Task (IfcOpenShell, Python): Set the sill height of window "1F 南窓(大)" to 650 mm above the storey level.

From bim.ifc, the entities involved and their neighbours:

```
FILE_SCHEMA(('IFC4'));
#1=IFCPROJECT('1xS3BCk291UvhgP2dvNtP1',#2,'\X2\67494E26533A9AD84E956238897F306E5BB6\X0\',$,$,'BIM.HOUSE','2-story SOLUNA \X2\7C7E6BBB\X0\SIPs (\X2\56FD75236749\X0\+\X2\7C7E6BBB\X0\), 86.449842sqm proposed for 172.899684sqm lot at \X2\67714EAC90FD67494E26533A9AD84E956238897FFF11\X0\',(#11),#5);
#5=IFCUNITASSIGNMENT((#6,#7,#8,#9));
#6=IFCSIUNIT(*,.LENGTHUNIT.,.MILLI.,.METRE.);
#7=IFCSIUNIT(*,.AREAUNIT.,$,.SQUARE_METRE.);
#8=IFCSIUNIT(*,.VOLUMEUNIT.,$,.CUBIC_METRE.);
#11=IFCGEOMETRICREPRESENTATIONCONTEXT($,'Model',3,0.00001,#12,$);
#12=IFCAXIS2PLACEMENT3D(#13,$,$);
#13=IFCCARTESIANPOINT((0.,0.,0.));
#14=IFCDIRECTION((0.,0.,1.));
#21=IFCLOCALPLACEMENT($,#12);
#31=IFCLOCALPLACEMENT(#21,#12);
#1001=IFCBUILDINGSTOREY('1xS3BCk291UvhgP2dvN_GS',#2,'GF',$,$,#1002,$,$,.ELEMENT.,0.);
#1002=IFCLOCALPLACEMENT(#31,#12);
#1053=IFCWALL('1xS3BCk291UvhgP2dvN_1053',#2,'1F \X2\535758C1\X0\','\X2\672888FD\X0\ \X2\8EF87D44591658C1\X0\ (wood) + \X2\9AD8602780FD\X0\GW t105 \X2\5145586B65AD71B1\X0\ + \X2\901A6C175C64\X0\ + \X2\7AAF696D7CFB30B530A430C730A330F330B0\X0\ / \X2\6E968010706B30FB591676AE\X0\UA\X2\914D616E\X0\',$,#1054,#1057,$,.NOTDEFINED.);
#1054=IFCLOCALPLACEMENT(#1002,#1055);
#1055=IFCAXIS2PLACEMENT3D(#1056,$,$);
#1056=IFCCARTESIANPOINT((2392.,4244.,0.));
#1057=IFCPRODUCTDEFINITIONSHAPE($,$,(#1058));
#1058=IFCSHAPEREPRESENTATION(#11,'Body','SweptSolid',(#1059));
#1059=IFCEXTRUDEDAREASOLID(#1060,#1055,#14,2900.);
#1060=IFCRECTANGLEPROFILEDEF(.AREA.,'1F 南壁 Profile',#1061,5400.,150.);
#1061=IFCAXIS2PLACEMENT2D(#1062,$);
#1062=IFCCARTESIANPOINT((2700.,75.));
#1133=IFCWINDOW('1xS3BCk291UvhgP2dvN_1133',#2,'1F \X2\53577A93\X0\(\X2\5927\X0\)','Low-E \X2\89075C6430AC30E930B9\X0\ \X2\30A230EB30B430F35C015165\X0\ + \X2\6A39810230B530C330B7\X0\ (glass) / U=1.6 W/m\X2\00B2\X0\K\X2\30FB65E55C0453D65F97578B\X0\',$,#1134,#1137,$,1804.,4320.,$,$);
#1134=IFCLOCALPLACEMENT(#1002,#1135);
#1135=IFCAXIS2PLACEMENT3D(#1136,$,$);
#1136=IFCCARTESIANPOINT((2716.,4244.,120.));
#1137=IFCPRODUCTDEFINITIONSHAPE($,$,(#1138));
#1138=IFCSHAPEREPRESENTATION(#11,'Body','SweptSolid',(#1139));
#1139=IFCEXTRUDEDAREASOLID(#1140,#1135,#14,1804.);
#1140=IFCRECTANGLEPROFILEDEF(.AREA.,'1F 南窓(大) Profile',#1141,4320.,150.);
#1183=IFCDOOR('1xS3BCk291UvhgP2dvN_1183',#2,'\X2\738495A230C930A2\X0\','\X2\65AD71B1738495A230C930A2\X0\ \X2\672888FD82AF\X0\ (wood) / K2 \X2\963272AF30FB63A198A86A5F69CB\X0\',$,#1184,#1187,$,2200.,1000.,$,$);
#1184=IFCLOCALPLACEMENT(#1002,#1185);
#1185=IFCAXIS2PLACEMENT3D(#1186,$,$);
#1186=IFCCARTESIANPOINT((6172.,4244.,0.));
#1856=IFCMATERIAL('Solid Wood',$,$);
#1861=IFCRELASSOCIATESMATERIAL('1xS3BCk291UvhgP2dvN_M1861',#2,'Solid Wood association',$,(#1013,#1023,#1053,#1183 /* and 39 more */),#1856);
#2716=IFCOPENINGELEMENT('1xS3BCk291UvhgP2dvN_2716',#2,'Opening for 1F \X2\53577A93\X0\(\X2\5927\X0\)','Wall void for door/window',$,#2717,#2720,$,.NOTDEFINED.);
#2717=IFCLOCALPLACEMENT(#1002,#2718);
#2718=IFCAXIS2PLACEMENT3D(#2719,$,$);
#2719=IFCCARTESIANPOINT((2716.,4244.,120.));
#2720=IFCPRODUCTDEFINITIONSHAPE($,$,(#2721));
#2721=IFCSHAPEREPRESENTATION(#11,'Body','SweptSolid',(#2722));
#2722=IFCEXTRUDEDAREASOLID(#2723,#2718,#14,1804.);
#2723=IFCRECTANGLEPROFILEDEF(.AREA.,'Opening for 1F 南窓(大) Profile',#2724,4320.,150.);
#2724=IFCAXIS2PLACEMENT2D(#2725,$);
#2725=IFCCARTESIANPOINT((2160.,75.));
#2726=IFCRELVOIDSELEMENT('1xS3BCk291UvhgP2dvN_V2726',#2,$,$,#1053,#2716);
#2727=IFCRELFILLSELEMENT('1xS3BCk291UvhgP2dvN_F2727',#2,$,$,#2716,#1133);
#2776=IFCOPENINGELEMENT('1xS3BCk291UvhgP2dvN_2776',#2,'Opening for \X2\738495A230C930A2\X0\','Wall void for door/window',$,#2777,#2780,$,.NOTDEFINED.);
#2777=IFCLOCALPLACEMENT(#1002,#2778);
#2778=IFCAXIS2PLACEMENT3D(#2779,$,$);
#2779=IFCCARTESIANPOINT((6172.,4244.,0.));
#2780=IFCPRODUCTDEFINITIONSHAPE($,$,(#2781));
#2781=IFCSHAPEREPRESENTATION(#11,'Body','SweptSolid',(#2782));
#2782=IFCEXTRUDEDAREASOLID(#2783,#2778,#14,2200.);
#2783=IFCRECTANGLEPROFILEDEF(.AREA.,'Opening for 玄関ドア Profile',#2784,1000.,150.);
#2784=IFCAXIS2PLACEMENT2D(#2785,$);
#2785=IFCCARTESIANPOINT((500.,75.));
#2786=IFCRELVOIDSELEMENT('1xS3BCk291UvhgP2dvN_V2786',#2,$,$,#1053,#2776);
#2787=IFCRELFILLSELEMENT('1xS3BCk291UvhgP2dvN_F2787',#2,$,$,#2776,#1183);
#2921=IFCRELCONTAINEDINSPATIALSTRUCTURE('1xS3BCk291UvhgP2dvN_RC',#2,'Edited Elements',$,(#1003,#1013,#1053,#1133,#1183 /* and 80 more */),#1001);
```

```python
import numpy as np
import ifcopenshell
import ifcopenshell.api.geometry
import ifcopenshell.geom
import ifcopenshell.util.element
import ifcopenshell.util.placement
import ifcopenshell.util.shape
import ifcopenshell.util.unit

model = ifcopenshell.open("bim.ifc")
unit_scale = ifcopenshell.util.unit.calculate_unit_scale(model)

window = model.by_guid("1xS3BCk291UvhgP2dvN_1133")
opening = window.FillsVoids[0].RelatingOpeningElement
storey = ifcopenshell.util.element.get_container(window, ifc_class="IfcBuildingStorey")
level = ifcopenshell.util.placement.get_local_placement(storey.ObjectPlacement)[2, 3]

# The opening's origin need not be at the sill, so measure its lowest point.
shape = ifcopenshell.geom.create_shape(ifcopenshell.geom.settings(), opening)
bottom = ifcopenshell.util.shape.get_shape_bottom_elevation(shape, shape.geometry) / unit_scale
dz = level + 0.65 / unit_scale - bottom

shift = np.array([0.0, 0.0, dz])
# The window is not placed relative to its opening, so move both.
for product in (opening, window):
    matrix = ifcopenshell.util.placement.get_local_placement(product.ObjectPlacement)
    matrix[:3, 3] += shift
    ifcopenshell.api.geometry.edit_object_placement(model, product=product, matrix=matrix, is_si=False)

print(f"moved by {dz * unit_scale:+.3f} m")

model.write("bim-out.ifc")
```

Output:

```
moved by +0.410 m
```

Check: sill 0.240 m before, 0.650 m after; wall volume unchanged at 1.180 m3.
